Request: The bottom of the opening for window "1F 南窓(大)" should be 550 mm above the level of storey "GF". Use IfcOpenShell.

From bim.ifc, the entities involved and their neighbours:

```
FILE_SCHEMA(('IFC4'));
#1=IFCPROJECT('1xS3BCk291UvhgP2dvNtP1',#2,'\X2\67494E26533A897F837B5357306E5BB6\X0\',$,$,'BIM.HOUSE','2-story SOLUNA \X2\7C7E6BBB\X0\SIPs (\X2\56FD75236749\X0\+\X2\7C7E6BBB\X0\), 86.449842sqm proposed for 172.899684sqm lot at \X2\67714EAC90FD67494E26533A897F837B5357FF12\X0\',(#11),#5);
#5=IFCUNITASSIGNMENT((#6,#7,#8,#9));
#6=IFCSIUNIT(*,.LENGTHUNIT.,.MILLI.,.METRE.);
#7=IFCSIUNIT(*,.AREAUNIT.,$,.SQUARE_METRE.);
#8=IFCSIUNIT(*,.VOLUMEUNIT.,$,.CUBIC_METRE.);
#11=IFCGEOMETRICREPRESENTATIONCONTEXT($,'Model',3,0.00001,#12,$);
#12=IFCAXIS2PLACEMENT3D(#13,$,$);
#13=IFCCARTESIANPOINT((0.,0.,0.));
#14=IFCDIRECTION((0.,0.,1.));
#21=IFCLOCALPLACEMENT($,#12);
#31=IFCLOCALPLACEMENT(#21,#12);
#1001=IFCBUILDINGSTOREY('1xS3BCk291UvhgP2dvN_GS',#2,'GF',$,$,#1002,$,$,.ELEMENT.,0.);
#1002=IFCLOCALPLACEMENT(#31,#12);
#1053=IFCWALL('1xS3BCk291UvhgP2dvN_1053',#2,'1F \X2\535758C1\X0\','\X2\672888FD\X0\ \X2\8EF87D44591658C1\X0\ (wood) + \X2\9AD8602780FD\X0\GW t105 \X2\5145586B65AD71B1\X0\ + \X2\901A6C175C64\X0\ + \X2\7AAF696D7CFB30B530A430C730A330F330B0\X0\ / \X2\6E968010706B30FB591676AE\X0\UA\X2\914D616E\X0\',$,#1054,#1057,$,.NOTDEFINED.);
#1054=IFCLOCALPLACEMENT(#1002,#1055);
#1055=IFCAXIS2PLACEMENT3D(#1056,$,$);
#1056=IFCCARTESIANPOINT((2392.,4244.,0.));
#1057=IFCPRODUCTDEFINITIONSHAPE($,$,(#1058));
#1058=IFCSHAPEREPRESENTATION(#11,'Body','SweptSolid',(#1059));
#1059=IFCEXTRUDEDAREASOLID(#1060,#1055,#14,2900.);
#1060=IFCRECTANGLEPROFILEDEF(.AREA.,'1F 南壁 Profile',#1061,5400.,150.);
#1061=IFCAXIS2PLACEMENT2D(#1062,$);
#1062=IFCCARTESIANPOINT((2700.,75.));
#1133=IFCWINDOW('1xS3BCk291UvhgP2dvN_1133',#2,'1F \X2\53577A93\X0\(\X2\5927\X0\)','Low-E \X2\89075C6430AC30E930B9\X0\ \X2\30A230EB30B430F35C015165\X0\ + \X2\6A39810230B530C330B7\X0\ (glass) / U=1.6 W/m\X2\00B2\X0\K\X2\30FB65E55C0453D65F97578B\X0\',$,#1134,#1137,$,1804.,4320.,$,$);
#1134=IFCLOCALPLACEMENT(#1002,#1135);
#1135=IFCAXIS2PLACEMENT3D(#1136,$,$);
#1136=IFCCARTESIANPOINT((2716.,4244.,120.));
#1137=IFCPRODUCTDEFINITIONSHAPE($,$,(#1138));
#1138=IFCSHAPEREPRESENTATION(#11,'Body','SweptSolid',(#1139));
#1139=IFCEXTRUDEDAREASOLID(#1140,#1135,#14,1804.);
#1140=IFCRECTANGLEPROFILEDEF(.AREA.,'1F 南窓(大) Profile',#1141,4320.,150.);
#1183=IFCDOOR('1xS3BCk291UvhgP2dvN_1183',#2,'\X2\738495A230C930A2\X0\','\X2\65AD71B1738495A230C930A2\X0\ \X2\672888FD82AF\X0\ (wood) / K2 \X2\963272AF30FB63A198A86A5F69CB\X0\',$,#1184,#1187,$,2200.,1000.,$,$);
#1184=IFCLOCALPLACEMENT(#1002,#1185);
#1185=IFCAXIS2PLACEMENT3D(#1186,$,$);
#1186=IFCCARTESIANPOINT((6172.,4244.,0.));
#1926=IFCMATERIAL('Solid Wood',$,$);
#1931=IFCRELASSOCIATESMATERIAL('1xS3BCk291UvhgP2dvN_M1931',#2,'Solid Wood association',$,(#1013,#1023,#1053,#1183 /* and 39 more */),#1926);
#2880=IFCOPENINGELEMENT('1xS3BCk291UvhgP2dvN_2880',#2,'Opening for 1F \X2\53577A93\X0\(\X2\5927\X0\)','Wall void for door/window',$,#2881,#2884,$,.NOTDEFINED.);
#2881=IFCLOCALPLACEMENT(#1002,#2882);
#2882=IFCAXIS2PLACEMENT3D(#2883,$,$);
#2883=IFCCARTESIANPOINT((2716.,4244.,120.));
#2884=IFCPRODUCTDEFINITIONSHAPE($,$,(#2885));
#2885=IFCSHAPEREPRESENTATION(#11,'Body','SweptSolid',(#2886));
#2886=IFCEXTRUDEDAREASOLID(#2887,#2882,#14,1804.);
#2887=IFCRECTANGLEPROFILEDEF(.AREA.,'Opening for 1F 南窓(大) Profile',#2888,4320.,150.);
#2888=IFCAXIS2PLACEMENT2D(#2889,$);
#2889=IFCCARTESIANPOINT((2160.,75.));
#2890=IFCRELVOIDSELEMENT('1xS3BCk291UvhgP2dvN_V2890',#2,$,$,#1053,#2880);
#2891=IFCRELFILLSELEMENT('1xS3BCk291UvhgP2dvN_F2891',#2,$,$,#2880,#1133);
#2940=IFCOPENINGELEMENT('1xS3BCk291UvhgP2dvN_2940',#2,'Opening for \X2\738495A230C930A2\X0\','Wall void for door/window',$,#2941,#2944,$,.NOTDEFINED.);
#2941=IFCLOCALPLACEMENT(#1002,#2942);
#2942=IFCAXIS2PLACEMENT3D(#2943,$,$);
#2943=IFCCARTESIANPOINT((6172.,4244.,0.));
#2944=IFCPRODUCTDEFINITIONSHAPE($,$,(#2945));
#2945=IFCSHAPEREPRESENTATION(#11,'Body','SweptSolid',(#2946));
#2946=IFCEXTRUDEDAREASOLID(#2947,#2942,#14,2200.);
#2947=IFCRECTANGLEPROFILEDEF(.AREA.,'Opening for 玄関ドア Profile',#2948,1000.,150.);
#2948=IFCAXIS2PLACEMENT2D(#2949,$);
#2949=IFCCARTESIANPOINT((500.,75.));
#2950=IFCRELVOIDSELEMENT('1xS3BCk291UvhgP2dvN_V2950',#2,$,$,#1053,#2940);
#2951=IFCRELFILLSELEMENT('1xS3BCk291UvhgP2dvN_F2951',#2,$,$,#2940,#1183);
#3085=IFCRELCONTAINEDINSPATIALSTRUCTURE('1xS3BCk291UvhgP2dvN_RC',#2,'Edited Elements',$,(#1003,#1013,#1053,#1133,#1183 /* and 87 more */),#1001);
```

```python
import numpy as np
import ifcopenshell
import ifcopenshell.api.geometry
import ifcopenshell.geom
import ifcopenshell.util.element
import ifcopenshell.util.placement
import ifcopenshell.util.shape
import ifcopenshell.util.unit

model = ifcopenshell.open("bim.ifc")
unit_scale = ifcopenshell.util.unit.calculate_unit_scale(model)

window = model.by_guid("1xS3BCk291UvhgP2dvN_1133")
opening = window.FillsVoids[0].RelatingOpeningElement
storey = ifcopenshell.util.element.get_container(window, ifc_class="IfcBuildingStorey")
level = ifcopenshell.util.placement.get_local_placement(storey.ObjectPlacement)[2, 3]

# The opening's origin need not be at the sill, so measure its lowest point.
shape = ifcopenshell.geom.create_shape(ifcopenshell.geom.settings(), opening)
bottom = ifcopenshell.util.shape.get_shape_bottom_elevation(shape, shape.geometry) / unit_scale
dz = level + 0.55 / unit_scale - bottom

shift = np.array([0.0, 0.0, dz])
# The window is not placed relative to its opening, so move both.
for product in (opening, window):
    matrix = ifcopenshell.util.placement.get_local_placement(product.ObjectPlacement)
    matrix[:3, 3] += shift
    ifcopenshell.api.geometry.edit_object_placement(model, product=product, matrix=matrix, is_si=False)

print(f"moved by {dz * unit_scale:+.3f} m")

model.write("bim_updated.ifc")
```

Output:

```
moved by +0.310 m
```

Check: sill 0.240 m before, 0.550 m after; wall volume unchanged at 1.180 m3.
